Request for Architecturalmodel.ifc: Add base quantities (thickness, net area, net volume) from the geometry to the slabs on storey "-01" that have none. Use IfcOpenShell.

First a look at what the model holds.

```python
import ifcopenshell
import ifcopenshell.util.element
import ifcopenshell.util.unit

model = ifcopenshell.open("Architecturalmodel.ifc")
print(model.schema)
for unit_type in ("LENGTHUNIT", "AREAUNIT", "VOLUMEUNIT"):
    print(unit_type, ifcopenshell.util.unit.calculate_unit_scale(model, unit_type))
storey = next(s for s in model.by_type("IfcBuildingStorey") if s.Name == "-01")
slabs = [e for e in ifcopenshell.util.element.get_decomposition(storey) if e.is_a("IfcSlab")]
for e in sorted(slabs, key=lambda e: e.id()):
    print(e.id(), e.is_a(), e.Name, list(ifcopenshell.util.element.get_psets(e, qtos_only=True)), sep=" | ")
```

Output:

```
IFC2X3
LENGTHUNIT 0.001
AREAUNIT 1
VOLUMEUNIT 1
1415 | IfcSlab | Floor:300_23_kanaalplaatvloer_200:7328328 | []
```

```python
import ifcopenshell
import ifcopenshell.api.pset
import ifcopenshell.geom
import ifcopenshell.util.element
import ifcopenshell.util.shape
import ifcopenshell.util.unit

model = ifcopenshell.open("Architecturalmodel.ifc")
unit_scale = ifcopenshell.util.unit.calculate_unit_scale(model)
area_scale = ifcopenshell.util.unit.calculate_unit_scale(model, "AREAUNIT")
volume_scale = ifcopenshell.util.unit.calculate_unit_scale(model, "VOLUMEUNIT")
settings = ifcopenshell.geom.settings()

storey = next(s for s in model.by_type("IfcBuildingStorey") if s.Name == "-01")
slabs = [e for e in ifcopenshell.util.element.get_decomposition(storey) if e.is_a("IfcSlab")]

for e in sorted(slabs, key=lambda e: e.id()):
    if ifcopenshell.util.element.get_psets(e, qtos_only=True, should_inherit=False):
        continue
    # Geometry comes back in metres, in the element's own axes.
    shape = ifcopenshell.geom.create_shape(settings, e)
    values = {
        "Width": ifcopenshell.util.shape.get_z(shape.geometry) / unit_scale,
        "NetArea": ifcopenshell.util.shape.get_footprint_area(shape.geometry) / area_scale,
        "NetVolume": ifcopenshell.util.shape.get_volume(shape.geometry) / volume_scale,
    }
    qto = ifcopenshell.api.pset.add_qto(model, product=e, name="BaseQuantities")
    ifcopenshell.api.pset.edit_qto(model, qto=qto, properties=values)
    print(e.id(), {k: round(v, 3) for k, v in values.items()})

model.write("Architecturalmodel_rev.ifc")
```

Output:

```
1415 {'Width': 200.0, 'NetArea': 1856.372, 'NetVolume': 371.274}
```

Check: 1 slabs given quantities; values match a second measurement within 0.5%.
